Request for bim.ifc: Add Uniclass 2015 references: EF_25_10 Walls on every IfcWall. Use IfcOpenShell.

First a look at what the model holds.

```python
import ifcopenshell

model = ifcopenshell.open("bim.ifc")
print(model.schema)
print("classifications:", [c.Name for c in model.by_type("IfcClassification")])
for ifc_class in ("IfcDoor", "IfcRoof", "IfcStair", "IfcWall", "IfcWindow"):
    print(ifc_class, len(model.by_type(ifc_class)))
```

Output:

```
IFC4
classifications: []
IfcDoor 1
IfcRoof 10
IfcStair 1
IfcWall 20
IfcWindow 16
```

```python
import ifcopenshell
import ifcopenshell.api.classification

model = ifcopenshell.open("bim.ifc")

system = ifcopenshell.api.classification.add_classification(model, classification="Uniclass 2015")

codes = {
    "IfcWall": ("EF_25_10", "Walls"),
}
for ifc_class, (code, name) in codes.items():
    products = model.by_type(ifc_class)
    ifcopenshell.api.classification.add_reference(
        model, products=products, classification=system, identification=code, name=name
    )
    print(code, len(products))

model.write("bim_edited.ifc")
```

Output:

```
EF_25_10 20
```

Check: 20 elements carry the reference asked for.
